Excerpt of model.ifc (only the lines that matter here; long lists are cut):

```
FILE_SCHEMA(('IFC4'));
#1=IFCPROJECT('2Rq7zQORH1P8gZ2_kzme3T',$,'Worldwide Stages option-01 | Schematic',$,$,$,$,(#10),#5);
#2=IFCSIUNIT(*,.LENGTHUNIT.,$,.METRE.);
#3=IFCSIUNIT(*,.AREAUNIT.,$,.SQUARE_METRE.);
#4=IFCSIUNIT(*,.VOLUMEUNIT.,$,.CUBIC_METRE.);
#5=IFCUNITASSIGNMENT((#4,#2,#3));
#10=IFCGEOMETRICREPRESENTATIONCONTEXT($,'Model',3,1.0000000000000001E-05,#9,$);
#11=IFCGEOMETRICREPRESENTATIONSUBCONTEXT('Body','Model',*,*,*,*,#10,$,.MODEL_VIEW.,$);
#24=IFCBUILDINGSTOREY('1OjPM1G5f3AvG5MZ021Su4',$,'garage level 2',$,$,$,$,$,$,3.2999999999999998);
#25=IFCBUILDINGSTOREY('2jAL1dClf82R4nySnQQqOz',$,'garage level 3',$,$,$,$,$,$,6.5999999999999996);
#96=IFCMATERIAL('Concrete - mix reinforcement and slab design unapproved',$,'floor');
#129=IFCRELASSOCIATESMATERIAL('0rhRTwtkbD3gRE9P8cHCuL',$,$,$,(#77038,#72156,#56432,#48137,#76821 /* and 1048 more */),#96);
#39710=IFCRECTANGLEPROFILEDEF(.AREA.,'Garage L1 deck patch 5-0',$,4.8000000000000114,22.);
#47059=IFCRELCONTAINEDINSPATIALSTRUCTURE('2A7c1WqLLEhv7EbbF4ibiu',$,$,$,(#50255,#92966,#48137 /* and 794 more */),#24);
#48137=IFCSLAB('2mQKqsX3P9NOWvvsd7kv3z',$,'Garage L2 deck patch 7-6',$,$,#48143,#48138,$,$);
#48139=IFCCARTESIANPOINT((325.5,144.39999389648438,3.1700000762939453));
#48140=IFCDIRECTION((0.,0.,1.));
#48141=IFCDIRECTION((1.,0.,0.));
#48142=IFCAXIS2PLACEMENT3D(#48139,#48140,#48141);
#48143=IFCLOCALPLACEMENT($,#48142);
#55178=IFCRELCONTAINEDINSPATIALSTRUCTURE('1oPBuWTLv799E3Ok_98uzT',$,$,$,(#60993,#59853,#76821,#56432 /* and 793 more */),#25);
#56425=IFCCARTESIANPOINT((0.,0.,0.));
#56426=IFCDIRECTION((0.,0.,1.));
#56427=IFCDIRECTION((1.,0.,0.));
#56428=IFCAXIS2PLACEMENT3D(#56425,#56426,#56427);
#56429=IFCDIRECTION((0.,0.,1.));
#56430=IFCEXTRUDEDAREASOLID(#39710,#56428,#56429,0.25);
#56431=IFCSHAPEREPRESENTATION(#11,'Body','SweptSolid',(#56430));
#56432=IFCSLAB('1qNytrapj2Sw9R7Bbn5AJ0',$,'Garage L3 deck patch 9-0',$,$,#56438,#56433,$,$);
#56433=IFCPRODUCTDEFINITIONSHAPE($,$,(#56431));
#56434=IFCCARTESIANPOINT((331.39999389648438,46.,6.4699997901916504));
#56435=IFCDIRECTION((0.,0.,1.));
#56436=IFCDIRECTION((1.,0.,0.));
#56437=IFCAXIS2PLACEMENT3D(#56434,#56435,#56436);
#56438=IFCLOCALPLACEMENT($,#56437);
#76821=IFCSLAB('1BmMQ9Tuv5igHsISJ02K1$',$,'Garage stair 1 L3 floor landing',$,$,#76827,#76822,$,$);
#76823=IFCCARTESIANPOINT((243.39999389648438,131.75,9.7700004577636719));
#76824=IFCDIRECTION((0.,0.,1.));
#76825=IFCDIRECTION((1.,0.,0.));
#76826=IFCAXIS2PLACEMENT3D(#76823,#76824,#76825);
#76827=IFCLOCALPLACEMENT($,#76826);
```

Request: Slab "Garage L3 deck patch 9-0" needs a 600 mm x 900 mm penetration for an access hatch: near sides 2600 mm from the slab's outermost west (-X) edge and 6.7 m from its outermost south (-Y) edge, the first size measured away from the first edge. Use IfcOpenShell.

```python
import numpy as np
import ifcopenshell
import ifcopenshell.api.feature
import ifcopenshell.api.geometry
import ifcopenshell.api.root
import ifcopenshell.geom
import ifcopenshell.util.placement
import ifcopenshell.util.representation
import ifcopenshell.util.shape
import ifcopenshell.util.unit

model = ifcopenshell.open("model.ifc")
unit_scale = ifcopenshell.util.unit.calculate_unit_scale(model)
settings = ifcopenshell.geom.settings()


def volume(element):
    """Net volume in cubic metres, openings subtracted."""
    shape = ifcopenshell.geom.create_shape(settings, element)
    return ifcopenshell.util.shape.get_volume(shape.geometry)


slab = model.by_guid("1qNytrapj2Sw9R7Bbn5AJ0")
before = volume(slab)

# Extent in the slab's own axes, in metres. The edges named are its -X and -Y sides.
slab_shape = ifcopenshell.geom.create_shape(settings, slab)
vertices = ifcopenshell.util.shape.get_vertices(slab_shape.geometry)
x_min, y_min, bottom = vertices.min(axis=0)
top = vertices[:, 2].max()

opening = ifcopenshell.api.root.create_entity(model, ifc_class="IfcOpeningElement", name="Access hatch opening", predefined_type="OPENING")
context = ifcopenshell.util.representation.get_context(model, "Model", "Body", "MODEL_VIEW")
width, depth = 0.6, 0.9
outline = [(0.0, 0.0), (width, 0.0), (width, depth), (0.0, depth), (0.0, 0.0)]
# Overshoot both faces by 50 mm so the cut is clean.
shape = ifcopenshell.api.geometry.add_slab_representation(
    model, context=context, depth=top - bottom + 0.1, polyline=outline
)
ifcopenshell.api.geometry.assign_representation(model, product=opening, representation=shape)

matrix = ifcopenshell.util.placement.get_local_placement(slab.ObjectPlacement)
matrix[:, 3] = matrix @ np.append(np.array([x_min + 2.6, y_min + 6.7, bottom - 0.05]) / unit_scale, 1.0)
ifcopenshell.api.geometry.edit_object_placement(model, product=opening, matrix=matrix, is_si=False)
ifcopenshell.api.feature.add_feature(model, feature=opening, element=slab)

after = volume(slab)

print(f"slab volume {before:.3f} -> {after:.3f} m3")

model.write("model_updated.ifc")
```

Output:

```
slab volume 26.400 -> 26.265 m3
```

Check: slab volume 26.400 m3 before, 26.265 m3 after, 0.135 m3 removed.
